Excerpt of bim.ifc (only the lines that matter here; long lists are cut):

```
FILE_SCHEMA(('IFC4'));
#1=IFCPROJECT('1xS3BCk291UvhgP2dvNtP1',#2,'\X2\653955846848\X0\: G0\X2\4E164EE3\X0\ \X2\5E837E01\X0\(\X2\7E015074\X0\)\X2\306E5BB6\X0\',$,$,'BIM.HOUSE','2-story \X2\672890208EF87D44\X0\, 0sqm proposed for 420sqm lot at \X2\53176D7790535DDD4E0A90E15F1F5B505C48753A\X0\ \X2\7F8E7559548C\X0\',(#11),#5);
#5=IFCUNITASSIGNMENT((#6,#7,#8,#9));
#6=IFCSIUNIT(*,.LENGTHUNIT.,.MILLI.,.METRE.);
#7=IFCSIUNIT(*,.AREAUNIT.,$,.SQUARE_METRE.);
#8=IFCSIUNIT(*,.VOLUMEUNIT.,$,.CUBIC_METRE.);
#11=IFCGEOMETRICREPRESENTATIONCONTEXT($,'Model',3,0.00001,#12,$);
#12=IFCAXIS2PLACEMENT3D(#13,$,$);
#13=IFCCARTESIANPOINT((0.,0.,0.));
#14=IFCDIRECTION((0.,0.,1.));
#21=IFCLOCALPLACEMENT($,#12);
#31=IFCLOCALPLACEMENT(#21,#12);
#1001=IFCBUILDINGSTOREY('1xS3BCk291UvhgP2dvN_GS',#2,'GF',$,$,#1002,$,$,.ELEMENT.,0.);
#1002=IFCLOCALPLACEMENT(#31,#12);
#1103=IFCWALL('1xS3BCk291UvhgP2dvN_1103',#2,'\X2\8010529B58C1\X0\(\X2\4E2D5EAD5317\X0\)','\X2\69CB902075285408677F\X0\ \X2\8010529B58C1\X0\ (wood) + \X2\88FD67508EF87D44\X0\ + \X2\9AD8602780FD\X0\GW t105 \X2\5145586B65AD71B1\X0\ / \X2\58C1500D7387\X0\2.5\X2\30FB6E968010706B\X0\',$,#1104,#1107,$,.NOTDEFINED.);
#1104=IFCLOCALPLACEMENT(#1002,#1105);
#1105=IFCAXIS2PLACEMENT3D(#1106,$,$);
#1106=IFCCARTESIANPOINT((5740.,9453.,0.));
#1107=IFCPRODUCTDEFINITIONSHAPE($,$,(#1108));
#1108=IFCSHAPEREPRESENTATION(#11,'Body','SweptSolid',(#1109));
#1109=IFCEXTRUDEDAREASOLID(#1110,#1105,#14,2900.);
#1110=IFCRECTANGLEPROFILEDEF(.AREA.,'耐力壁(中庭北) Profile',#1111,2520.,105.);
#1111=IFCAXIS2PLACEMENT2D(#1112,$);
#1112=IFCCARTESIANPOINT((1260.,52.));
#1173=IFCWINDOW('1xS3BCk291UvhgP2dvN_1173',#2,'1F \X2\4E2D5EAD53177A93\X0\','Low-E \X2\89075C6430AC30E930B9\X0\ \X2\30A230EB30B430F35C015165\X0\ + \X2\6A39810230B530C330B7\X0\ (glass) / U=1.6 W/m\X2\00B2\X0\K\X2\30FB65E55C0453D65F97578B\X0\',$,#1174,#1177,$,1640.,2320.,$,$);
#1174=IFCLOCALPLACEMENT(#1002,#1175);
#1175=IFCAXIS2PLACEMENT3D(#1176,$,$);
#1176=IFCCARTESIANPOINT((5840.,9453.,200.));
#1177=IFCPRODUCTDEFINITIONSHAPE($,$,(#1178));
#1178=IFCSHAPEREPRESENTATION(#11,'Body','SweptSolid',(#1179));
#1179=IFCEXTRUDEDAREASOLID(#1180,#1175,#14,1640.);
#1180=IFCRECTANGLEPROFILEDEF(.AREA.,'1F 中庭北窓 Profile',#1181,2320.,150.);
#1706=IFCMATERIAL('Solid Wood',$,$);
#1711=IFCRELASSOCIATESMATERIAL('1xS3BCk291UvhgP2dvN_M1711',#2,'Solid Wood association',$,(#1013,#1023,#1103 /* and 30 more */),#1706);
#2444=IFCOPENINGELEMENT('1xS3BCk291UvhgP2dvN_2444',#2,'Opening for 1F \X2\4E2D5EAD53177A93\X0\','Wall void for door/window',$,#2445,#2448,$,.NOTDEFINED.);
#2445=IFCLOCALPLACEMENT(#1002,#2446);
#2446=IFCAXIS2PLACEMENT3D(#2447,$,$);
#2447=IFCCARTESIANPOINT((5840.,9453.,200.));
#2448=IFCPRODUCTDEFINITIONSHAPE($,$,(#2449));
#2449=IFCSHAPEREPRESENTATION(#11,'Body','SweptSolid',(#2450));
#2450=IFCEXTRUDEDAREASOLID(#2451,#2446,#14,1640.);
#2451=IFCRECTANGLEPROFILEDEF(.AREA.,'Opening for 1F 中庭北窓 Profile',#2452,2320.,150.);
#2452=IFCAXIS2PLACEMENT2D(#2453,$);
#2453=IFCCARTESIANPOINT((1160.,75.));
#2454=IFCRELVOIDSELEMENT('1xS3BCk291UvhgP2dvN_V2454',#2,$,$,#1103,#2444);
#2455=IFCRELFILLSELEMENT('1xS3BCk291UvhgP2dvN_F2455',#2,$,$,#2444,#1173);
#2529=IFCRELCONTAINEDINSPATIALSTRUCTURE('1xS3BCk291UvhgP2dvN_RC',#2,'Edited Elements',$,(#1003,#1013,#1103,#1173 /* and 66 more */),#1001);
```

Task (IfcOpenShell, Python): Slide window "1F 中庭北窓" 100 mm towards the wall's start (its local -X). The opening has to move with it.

```python
import ifcopenshell
import ifcopenshell.api.geometry
import ifcopenshell.util.placement

model = ifcopenshell.open("bim.ifc")

window = model.by_guid("1xS3BCk291UvhgP2dvN_1173")
opening = window.FillsVoids[0].RelatingOpeningElement
wall = opening.VoidsElements[0].RelatingBuildingElement

wall_matrix = ifcopenshell.util.placement.get_local_placement(wall.ObjectPlacement)
shift = wall_matrix[:3, 0] * -100.0
before = ifcopenshell.util.placement.get_local_placement(window.ObjectPlacement)[:3, 3].copy()

# The window is not placed relative to its opening, so move both.
for product in (opening, window):
    matrix = ifcopenshell.util.placement.get_local_placement(product.ObjectPlacement)
    matrix[:3, 3] += shift
    ifcopenshell.api.geometry.edit_object_placement(model, product=product, matrix=matrix, is_si=False)

after = ifcopenshell.util.placement.get_local_placement(window.ObjectPlacement)[:3, 3]
print("window moved by", (after - before).round(3) + 0.0)

model.write("bim_rev.ifc")
```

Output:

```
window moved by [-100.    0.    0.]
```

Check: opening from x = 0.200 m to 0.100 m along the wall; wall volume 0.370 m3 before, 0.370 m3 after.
